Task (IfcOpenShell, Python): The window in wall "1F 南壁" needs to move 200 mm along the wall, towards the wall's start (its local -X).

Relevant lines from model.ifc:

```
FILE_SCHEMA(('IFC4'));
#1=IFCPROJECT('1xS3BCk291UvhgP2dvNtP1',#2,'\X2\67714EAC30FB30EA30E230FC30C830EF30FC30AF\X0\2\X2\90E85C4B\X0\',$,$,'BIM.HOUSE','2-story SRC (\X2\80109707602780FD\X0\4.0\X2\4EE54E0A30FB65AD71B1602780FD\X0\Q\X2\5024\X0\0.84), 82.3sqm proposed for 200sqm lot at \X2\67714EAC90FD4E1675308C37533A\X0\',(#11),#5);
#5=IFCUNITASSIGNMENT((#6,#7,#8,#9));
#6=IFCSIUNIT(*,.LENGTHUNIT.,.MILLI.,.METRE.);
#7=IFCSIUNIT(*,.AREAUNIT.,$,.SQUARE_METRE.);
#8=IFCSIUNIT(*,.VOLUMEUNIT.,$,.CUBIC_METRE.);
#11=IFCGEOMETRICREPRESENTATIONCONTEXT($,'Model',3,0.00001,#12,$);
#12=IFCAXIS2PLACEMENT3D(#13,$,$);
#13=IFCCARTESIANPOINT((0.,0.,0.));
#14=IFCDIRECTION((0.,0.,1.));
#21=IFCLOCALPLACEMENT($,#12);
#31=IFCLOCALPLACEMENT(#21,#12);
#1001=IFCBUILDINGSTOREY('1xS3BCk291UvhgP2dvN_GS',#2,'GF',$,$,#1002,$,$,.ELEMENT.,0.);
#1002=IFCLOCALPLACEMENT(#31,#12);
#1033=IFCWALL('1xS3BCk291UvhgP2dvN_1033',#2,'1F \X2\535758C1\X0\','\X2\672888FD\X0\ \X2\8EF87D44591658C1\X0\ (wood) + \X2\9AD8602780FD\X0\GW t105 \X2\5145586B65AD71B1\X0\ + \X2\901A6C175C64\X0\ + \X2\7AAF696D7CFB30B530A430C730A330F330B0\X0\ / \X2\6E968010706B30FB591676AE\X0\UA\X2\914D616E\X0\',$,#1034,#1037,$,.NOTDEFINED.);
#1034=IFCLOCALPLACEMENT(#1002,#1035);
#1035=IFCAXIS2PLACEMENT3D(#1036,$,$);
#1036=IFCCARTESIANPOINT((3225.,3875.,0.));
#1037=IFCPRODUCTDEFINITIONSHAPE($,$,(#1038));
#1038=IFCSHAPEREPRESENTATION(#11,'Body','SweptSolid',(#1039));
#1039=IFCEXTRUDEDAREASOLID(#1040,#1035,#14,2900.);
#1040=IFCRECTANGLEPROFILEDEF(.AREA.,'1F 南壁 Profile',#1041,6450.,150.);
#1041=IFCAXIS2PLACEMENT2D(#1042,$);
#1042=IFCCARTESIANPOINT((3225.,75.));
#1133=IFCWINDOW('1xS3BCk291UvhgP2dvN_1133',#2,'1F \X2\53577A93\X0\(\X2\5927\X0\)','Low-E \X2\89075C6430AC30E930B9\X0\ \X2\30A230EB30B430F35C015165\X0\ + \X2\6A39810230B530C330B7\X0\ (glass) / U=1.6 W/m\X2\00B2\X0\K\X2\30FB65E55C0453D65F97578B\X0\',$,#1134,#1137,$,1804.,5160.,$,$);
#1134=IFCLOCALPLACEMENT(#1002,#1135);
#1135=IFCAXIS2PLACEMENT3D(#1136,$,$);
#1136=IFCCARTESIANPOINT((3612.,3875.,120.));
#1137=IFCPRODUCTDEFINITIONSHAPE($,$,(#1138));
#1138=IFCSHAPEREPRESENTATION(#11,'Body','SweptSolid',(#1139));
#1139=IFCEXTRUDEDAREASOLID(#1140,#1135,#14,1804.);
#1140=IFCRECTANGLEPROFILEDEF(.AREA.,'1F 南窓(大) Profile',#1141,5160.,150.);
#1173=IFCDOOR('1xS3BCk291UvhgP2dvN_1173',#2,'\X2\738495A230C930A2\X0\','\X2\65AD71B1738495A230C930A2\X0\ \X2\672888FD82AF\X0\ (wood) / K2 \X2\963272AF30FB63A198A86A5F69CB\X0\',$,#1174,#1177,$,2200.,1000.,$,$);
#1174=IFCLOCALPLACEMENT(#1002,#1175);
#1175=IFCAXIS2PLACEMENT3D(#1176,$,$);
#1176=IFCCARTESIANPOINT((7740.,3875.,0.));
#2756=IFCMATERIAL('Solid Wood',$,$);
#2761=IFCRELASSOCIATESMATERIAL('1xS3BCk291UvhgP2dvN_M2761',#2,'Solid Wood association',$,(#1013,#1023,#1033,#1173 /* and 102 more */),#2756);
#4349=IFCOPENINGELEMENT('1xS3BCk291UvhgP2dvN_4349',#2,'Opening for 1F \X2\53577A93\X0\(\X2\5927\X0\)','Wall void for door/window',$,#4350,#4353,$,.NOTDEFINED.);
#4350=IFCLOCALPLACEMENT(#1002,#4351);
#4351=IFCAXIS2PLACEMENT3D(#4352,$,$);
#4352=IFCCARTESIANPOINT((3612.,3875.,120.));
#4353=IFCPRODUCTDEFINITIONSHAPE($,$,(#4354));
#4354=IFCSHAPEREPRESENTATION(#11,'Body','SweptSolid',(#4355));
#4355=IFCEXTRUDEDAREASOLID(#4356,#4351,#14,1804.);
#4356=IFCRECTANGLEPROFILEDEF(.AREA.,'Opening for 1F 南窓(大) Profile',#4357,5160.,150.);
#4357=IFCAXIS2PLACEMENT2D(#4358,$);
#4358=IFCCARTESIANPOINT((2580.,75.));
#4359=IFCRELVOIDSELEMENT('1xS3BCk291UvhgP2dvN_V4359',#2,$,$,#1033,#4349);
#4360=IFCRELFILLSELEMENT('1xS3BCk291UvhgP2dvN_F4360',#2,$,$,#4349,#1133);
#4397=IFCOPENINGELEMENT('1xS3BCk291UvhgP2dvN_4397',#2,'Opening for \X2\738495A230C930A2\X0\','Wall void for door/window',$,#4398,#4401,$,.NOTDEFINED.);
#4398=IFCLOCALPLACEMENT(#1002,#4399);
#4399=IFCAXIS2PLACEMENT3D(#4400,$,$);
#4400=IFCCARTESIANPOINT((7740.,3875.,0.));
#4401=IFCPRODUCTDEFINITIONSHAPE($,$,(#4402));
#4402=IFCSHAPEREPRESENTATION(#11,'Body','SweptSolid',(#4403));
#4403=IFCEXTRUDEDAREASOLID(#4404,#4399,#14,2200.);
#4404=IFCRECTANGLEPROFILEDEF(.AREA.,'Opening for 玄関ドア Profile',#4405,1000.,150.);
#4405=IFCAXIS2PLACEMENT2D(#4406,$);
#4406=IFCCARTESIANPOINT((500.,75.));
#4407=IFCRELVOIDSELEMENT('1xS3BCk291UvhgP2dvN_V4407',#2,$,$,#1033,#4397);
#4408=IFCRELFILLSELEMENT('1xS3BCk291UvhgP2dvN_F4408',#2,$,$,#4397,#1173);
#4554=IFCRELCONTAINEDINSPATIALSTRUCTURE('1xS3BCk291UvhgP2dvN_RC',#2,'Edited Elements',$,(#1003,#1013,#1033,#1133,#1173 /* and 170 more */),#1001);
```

```python
import ifcopenshell
import ifcopenshell.api.geometry
import ifcopenshell.util.placement
import ifcopenshell.util.unit

model = ifcopenshell.open("model.ifc")
unit_scale = ifcopenshell.util.unit.calculate_unit_scale(model)

window = model.by_guid("1xS3BCk291UvhgP2dvN_1133")
opening = window.FillsVoids[0].RelatingOpeningElement
wall = opening.VoidsElements[0].RelatingBuildingElement

wall_matrix = ifcopenshell.util.placement.get_local_placement(wall.ObjectPlacement)
shift = wall_matrix[:3, 0] * -0.2 / unit_scale
before = ifcopenshell.util.placement.get_local_placement(window.ObjectPlacement)[:3, 3].copy()

# The window is not placed relative to its opening, so move both.
for product in (opening, window):
    matrix = ifcopenshell.util.placement.get_local_placement(product.ObjectPlacement)
    matrix[:3, 3] += shift
    ifcopenshell.api.geometry.edit_object_placement(model, product=product, matrix=matrix, is_si=False)

after = ifcopenshell.util.placement.get_local_placement(window.ObjectPlacement)[:3, 3]
print("window moved by", (after - before).round(3) + 0.0)

model.write("model_updated.ifc")
```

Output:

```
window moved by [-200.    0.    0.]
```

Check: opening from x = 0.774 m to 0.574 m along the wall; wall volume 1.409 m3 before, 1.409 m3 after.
